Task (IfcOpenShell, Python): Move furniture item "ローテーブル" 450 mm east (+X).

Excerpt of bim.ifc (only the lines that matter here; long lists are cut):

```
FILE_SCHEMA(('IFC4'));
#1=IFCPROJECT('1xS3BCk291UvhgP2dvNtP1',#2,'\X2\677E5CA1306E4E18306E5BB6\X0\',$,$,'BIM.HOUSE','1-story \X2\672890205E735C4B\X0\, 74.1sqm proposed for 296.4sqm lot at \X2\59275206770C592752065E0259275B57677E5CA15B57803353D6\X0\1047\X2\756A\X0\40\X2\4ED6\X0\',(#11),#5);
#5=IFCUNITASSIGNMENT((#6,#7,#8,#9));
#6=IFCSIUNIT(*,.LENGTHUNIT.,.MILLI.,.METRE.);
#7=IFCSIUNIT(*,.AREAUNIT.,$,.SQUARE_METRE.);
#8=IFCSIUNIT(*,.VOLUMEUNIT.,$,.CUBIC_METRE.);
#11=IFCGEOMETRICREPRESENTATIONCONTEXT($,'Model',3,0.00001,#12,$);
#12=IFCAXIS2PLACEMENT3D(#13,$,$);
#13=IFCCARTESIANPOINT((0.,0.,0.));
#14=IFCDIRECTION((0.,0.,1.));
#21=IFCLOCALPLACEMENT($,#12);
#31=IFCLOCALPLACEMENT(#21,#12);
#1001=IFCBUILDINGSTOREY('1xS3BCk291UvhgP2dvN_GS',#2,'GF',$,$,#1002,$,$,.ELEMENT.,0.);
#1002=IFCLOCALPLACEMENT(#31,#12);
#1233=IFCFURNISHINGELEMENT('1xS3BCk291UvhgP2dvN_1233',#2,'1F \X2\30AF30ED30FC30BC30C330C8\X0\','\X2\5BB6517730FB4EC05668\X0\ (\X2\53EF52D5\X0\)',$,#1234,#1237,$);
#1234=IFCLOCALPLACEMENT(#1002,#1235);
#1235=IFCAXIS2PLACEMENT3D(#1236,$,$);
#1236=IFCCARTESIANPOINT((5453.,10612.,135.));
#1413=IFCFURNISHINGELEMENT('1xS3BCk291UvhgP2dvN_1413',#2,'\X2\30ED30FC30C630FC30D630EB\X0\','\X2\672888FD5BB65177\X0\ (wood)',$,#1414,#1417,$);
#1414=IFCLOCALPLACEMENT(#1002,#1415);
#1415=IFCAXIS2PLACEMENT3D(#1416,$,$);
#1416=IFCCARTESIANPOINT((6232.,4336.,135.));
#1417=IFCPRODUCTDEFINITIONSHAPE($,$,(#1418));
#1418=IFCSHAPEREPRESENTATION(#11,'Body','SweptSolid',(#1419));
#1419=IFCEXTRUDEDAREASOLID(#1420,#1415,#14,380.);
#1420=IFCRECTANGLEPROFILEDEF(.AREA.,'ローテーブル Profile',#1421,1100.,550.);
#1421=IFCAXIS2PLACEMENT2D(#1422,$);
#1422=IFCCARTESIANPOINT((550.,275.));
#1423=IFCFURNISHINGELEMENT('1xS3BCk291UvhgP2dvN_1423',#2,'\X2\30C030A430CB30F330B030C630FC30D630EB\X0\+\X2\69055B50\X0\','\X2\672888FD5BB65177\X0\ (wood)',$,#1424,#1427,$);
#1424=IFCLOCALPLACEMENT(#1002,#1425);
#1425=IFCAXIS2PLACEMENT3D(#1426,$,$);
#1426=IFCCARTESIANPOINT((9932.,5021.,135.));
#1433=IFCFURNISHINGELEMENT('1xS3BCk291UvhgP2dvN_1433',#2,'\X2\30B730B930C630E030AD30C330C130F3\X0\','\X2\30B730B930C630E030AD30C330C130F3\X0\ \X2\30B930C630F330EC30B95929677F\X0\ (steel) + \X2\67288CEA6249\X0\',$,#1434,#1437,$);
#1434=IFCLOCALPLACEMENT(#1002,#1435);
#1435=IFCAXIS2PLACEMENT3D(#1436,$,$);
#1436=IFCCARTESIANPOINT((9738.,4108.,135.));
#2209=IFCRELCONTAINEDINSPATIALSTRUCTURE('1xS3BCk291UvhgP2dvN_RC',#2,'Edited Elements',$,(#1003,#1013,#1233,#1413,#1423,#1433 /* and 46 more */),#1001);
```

```python
import ifcopenshell
import ifcopenshell.api.geometry
import ifcopenshell.util.placement
import ifcopenshell.util.unit

model = ifcopenshell.open("bim.ifc")
unit_scale = ifcopenshell.util.unit.calculate_unit_scale(model)

item = model.by_guid("1xS3BCk291UvhgP2dvN_1413")
matrix = ifcopenshell.util.placement.get_local_placement(item.ObjectPlacement)
matrix[0, 3] += 0.45 / unit_scale
ifcopenshell.api.geometry.edit_object_placement(model, product=item, matrix=matrix, is_si=False)

print(ifcopenshell.util.placement.get_local_placement(item.ObjectPlacement).round(3) + 0.0)

model.write("bim_edited.ifc")
```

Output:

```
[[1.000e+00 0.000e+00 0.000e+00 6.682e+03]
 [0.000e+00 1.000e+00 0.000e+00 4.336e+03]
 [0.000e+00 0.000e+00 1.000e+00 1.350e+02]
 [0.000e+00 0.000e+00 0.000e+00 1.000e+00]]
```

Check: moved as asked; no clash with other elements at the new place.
